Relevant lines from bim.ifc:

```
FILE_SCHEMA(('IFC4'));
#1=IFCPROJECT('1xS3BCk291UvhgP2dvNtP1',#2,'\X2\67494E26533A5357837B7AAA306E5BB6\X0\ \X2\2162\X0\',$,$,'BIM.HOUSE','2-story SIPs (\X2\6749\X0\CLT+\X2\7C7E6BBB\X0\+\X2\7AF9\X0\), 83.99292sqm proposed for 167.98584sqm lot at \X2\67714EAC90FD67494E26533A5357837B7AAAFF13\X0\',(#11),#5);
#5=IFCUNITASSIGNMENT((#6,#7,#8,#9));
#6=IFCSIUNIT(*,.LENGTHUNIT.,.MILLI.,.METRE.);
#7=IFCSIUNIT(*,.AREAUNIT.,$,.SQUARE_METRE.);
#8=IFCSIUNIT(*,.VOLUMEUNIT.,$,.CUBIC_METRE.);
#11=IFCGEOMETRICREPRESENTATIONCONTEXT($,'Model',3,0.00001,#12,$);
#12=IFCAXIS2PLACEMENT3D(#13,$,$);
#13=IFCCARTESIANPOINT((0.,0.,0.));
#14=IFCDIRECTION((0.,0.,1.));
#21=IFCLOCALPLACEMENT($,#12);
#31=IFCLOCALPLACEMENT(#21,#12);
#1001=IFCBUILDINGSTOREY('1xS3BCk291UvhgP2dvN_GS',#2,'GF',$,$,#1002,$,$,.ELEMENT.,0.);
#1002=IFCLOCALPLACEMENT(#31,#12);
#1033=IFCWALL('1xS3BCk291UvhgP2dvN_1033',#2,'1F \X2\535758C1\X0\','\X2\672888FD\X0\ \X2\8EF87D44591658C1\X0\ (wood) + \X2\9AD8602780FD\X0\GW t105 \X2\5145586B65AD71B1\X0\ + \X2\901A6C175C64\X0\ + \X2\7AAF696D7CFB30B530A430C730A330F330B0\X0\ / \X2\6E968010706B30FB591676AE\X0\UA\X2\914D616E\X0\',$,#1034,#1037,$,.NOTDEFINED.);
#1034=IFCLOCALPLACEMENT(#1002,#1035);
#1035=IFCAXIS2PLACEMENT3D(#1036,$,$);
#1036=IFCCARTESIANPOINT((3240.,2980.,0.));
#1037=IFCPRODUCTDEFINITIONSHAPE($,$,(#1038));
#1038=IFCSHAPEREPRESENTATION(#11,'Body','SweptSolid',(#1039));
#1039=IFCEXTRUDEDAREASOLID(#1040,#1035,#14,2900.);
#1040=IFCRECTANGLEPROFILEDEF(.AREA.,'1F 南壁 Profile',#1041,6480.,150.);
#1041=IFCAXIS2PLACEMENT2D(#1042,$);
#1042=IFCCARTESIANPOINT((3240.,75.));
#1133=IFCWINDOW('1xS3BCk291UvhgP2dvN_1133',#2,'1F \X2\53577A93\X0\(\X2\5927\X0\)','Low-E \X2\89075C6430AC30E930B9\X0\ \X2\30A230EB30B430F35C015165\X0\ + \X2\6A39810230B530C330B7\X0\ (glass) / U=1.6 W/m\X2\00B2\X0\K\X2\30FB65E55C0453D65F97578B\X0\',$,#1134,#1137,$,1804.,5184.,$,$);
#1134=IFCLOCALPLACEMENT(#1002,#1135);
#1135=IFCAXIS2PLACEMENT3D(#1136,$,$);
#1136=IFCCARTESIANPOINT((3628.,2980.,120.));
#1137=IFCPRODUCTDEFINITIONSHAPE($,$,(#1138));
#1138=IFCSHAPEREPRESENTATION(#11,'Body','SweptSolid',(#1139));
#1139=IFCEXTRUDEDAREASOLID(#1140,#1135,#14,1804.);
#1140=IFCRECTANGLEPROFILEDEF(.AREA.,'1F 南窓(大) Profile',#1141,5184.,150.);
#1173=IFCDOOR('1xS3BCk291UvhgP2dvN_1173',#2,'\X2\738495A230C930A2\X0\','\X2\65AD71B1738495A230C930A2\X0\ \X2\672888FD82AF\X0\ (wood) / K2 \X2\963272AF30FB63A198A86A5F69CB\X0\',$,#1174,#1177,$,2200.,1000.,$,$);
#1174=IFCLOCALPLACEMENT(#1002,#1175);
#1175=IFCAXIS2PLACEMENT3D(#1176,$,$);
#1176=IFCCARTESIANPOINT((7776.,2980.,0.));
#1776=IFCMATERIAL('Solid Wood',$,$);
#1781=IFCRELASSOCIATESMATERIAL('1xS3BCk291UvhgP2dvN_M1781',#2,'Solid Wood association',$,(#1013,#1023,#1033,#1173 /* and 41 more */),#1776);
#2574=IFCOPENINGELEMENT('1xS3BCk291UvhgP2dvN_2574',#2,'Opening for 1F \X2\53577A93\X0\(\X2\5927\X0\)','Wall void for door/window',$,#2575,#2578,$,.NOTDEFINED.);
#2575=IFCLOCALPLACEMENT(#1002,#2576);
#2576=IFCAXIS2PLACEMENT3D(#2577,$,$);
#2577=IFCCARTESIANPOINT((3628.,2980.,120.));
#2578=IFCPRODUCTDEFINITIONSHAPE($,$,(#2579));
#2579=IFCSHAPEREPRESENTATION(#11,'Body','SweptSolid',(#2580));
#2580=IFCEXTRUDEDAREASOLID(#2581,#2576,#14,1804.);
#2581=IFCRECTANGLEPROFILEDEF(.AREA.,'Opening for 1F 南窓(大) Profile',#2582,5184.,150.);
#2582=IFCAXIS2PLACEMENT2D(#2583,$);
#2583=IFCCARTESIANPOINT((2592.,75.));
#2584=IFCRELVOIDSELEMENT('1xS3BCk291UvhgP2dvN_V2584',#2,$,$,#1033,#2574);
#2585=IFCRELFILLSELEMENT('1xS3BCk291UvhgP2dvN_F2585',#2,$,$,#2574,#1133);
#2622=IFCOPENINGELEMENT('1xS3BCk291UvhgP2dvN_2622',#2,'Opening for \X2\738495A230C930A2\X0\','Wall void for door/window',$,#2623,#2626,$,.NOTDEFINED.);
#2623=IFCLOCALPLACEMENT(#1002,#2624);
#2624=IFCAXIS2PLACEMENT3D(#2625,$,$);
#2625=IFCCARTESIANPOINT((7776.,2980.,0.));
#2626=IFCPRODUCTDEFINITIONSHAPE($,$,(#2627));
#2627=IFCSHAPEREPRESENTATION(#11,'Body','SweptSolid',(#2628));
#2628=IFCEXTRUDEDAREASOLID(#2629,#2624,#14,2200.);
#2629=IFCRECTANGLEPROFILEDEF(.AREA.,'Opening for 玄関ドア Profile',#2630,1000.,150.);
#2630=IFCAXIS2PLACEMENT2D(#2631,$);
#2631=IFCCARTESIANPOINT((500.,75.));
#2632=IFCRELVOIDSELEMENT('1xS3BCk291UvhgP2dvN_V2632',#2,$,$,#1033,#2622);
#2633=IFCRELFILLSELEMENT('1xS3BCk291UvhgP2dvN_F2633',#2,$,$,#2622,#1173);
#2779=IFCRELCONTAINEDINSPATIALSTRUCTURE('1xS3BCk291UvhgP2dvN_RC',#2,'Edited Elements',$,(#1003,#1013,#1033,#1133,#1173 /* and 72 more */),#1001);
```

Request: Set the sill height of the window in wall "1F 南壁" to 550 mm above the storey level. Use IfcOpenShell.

```python
import numpy as np
import ifcopenshell
import ifcopenshell.api.geometry
import ifcopenshell.geom
import ifcopenshell.util.element
import ifcopenshell.util.placement
import ifcopenshell.util.shape
import ifcopenshell.util.unit

model = ifcopenshell.open("bim.ifc")
unit_scale = ifcopenshell.util.unit.calculate_unit_scale(model)

window = model.by_id(1133)
opening = window.FillsVoids[0].RelatingOpeningElement
storey = ifcopenshell.util.element.get_container(window, ifc_class="IfcBuildingStorey")
level = ifcopenshell.util.placement.get_local_placement(storey.ObjectPlacement)[2, 3]

# The opening's origin need not be at the sill, so measure its lowest point.
shape = ifcopenshell.geom.create_shape(ifcopenshell.geom.settings(), opening)
bottom = ifcopenshell.util.shape.get_shape_bottom_elevation(shape, shape.geometry) / unit_scale
dz = level + 550.0 - bottom

shift = np.array([0.0, 0.0, dz])
# The window is not placed relative to its opening, so move both.
for product in (opening, window):
    matrix = ifcopenshell.util.placement.get_local_placement(product.ObjectPlacement)
    matrix[:3, 3] += shift
    ifcopenshell.api.geometry.edit_object_placement(model, product=product, matrix=matrix, is_si=False)

print(f"moved by {dz * unit_scale:+.3f} m")

model.write("bim-out.ifc")
```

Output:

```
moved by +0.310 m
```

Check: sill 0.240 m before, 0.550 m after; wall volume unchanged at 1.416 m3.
